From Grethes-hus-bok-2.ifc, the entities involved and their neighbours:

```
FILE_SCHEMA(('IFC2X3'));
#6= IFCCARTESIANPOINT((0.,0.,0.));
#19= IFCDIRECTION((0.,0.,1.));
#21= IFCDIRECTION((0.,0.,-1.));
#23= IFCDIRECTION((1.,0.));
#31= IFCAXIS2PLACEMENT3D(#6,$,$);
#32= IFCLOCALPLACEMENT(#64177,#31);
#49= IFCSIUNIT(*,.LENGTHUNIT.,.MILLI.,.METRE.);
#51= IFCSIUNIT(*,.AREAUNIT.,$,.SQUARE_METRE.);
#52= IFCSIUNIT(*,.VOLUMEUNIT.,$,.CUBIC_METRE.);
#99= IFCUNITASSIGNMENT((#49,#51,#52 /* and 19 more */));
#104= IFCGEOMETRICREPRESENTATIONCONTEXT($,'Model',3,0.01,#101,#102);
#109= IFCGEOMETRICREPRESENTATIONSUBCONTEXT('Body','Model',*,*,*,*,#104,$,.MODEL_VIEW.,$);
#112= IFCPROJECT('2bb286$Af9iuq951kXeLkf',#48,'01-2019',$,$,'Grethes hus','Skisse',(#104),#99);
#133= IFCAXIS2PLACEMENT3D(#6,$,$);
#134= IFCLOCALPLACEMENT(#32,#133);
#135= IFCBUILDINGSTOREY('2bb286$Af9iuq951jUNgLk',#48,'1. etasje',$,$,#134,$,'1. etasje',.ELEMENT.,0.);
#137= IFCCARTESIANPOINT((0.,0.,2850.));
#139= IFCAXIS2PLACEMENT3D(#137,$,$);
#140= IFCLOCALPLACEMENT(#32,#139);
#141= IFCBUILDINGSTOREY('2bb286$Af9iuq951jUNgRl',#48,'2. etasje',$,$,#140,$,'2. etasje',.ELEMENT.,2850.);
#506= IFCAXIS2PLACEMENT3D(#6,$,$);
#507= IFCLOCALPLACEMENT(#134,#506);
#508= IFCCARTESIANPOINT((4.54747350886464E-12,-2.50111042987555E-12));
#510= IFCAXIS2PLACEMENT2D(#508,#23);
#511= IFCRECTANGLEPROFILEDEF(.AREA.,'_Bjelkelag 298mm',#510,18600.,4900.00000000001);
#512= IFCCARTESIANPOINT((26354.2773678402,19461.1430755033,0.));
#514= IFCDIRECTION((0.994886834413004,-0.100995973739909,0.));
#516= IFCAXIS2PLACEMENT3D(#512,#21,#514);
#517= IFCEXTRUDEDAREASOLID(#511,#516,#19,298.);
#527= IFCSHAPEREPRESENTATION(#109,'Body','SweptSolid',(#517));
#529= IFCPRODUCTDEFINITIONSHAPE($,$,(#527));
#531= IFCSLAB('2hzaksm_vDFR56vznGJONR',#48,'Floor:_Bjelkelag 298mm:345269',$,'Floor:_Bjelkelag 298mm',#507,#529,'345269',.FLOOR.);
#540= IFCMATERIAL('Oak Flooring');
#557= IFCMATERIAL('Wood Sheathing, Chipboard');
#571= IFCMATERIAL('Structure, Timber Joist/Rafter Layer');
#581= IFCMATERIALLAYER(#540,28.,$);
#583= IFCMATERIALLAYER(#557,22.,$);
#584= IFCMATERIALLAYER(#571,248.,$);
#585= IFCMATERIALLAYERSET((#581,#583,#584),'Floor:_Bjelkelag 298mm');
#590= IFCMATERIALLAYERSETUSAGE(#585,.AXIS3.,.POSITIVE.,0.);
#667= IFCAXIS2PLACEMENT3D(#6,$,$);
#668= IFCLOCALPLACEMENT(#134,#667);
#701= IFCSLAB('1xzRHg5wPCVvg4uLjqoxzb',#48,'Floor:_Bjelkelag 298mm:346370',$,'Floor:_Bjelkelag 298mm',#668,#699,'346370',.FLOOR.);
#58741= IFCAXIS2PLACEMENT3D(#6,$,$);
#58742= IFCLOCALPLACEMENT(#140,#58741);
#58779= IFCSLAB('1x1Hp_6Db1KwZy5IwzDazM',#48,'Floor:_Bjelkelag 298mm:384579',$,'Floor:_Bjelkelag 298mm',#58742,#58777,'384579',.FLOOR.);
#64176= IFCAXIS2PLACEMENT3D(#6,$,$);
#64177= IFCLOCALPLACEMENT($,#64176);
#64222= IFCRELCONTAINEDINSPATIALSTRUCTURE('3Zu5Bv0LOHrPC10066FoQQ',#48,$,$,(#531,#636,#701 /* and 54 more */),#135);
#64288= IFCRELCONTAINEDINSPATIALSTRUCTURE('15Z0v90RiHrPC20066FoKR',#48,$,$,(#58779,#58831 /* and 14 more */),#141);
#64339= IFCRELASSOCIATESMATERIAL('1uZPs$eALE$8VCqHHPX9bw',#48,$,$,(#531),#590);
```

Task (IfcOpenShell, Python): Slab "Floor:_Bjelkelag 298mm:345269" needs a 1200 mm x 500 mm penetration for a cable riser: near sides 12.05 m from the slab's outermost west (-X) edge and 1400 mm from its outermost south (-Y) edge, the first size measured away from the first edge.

```python
import numpy as np
import ifcopenshell
import ifcopenshell.api.feature
import ifcopenshell.api.geometry
import ifcopenshell.api.root
import ifcopenshell.geom
import ifcopenshell.util.placement
import ifcopenshell.util.representation
import ifcopenshell.util.shape
import ifcopenshell.util.unit

model = ifcopenshell.open("Grethes-hus-bok-2.ifc")
unit_scale = ifcopenshell.util.unit.calculate_unit_scale(model)
settings = ifcopenshell.geom.settings()


def volume(element):
    """Net volume in cubic metres, openings subtracted."""
    shape = ifcopenshell.geom.create_shape(settings, element)
    return ifcopenshell.util.shape.get_volume(shape.geometry)


slab = model.by_id(531)
before = volume(slab)

# Extent in the slab's own axes, in metres. The edges named are its -X and -Y sides.
slab_shape = ifcopenshell.geom.create_shape(settings, slab)
vertices = ifcopenshell.util.shape.get_vertices(slab_shape.geometry)
x_min, y_min, bottom = vertices.min(axis=0)
top = vertices[:, 2].max()

opening = ifcopenshell.api.root.create_entity(model, ifc_class="IfcOpeningElement", name="Cable riser opening")
context = ifcopenshell.util.representation.get_context(model, "Model", "Body", "MODEL_VIEW")
width, depth = 1.2, 0.5
outline = [(0.0, 0.0), (width, 0.0), (width, depth), (0.0, depth), (0.0, 0.0)]
# Overshoot both faces by 50 mm so the cut is clean.
shape = ifcopenshell.api.geometry.add_slab_representation(
    model, context=context, depth=top - bottom + 0.1, polyline=outline
)
ifcopenshell.api.geometry.assign_representation(model, product=opening, representation=shape)

matrix = ifcopenshell.util.placement.get_local_placement(slab.ObjectPlacement)
matrix[:, 3] = matrix @ np.append(np.array([x_min + 12.05, y_min + 1.4, bottom - 0.05]) / unit_scale, 1.0)
ifcopenshell.api.geometry.edit_object_placement(model, product=opening, matrix=matrix, is_si=False)
ifcopenshell.api.feature.add_feature(model, feature=opening, element=slab)

after = volume(slab)

print(f"slab volume {before:.3f} -> {after:.3f} m3")

model.write("Grethes-hus-bok-2_v2.ifc")
```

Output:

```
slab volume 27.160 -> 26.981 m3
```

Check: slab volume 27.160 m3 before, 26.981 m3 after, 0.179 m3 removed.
